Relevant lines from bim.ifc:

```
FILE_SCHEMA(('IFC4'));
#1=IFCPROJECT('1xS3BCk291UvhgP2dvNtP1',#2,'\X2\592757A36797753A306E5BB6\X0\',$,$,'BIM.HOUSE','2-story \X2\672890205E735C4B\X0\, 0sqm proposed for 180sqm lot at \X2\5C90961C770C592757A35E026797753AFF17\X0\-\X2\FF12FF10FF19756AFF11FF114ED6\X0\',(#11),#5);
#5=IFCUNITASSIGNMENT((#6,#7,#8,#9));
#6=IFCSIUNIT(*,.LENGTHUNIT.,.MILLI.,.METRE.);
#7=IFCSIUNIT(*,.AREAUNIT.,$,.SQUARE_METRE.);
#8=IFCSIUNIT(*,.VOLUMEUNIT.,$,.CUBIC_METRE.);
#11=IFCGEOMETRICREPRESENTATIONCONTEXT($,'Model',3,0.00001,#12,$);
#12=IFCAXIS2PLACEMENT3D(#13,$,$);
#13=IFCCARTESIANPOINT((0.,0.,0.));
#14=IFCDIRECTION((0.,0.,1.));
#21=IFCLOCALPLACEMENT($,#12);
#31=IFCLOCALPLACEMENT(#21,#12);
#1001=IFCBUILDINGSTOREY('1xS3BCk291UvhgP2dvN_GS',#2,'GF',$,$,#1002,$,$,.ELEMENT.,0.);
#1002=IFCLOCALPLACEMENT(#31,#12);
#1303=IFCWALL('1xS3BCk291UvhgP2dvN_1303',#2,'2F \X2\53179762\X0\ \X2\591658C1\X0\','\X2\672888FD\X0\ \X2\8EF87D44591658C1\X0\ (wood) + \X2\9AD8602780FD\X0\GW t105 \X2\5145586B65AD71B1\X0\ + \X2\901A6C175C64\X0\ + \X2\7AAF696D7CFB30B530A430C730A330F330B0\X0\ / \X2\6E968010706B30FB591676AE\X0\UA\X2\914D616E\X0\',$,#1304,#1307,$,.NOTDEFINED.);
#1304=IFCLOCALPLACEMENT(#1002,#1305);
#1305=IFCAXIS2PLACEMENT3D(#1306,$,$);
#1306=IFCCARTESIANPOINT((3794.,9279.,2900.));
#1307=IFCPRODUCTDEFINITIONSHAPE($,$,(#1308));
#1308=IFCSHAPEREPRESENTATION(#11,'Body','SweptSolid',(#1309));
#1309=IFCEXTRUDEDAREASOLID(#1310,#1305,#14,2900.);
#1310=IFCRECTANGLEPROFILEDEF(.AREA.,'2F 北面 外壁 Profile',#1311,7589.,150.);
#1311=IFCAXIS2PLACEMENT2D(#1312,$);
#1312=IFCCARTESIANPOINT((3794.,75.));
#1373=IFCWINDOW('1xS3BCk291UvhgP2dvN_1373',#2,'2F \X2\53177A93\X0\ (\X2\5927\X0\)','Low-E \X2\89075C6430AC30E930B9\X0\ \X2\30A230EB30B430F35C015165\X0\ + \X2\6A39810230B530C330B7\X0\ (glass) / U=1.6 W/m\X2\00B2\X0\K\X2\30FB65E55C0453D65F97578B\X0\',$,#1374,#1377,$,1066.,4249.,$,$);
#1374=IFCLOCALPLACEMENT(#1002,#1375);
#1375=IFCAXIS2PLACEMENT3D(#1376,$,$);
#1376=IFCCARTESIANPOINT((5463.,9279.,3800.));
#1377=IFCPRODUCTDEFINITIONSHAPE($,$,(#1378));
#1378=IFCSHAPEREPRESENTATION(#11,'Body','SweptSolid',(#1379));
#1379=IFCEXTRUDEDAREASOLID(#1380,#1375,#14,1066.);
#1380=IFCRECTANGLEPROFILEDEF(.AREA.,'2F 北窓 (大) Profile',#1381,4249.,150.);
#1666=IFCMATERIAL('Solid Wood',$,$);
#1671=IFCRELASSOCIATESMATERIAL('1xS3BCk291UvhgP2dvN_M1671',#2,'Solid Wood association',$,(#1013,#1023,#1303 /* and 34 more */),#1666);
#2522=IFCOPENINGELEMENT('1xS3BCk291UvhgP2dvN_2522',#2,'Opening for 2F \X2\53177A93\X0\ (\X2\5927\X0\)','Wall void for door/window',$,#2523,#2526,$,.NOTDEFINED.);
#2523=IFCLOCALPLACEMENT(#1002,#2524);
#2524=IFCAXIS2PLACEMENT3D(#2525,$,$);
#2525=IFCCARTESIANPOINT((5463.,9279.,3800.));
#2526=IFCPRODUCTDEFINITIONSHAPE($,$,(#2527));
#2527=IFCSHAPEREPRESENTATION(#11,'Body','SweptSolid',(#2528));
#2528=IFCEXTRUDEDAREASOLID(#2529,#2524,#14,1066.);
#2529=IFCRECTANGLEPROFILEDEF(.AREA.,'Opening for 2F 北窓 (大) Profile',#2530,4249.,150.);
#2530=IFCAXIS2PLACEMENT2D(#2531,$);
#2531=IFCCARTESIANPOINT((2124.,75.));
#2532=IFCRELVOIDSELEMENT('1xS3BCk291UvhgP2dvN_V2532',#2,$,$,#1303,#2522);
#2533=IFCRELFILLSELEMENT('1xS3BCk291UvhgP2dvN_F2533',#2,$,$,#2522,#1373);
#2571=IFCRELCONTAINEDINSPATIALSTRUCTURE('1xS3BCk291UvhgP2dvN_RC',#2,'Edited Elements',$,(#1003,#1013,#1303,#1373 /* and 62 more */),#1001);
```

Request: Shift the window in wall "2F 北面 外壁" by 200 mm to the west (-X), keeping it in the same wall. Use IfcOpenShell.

```python
import ifcopenshell
import ifcopenshell.api.geometry
import ifcopenshell.util.placement

model = ifcopenshell.open("bim.ifc")

window = model.by_id(1373)
opening = window.FillsVoids[0].RelatingOpeningElement
wall = opening.VoidsElements[0].RelatingBuildingElement

wall_matrix = ifcopenshell.util.placement.get_local_placement(wall.ObjectPlacement)
shift = wall_matrix[:3, 0] * -200.0
before = ifcopenshell.util.placement.get_local_placement(window.ObjectPlacement)[:3, 3].copy()

# The window is not placed relative to its opening, so move both.
for product in (opening, window):
    matrix = ifcopenshell.util.placement.get_local_placement(product.ObjectPlacement)
    matrix[:3, 3] += shift
    ifcopenshell.api.geometry.edit_object_placement(model, product=product, matrix=matrix, is_si=False)

after = ifcopenshell.util.placement.get_local_placement(window.ObjectPlacement)[:3, 3]
print("window moved by", (after - before).round(3) + 0.0)

model.write("bim_rev.ifc")
```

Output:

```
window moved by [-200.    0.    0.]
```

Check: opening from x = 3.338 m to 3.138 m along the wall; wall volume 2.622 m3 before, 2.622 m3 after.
